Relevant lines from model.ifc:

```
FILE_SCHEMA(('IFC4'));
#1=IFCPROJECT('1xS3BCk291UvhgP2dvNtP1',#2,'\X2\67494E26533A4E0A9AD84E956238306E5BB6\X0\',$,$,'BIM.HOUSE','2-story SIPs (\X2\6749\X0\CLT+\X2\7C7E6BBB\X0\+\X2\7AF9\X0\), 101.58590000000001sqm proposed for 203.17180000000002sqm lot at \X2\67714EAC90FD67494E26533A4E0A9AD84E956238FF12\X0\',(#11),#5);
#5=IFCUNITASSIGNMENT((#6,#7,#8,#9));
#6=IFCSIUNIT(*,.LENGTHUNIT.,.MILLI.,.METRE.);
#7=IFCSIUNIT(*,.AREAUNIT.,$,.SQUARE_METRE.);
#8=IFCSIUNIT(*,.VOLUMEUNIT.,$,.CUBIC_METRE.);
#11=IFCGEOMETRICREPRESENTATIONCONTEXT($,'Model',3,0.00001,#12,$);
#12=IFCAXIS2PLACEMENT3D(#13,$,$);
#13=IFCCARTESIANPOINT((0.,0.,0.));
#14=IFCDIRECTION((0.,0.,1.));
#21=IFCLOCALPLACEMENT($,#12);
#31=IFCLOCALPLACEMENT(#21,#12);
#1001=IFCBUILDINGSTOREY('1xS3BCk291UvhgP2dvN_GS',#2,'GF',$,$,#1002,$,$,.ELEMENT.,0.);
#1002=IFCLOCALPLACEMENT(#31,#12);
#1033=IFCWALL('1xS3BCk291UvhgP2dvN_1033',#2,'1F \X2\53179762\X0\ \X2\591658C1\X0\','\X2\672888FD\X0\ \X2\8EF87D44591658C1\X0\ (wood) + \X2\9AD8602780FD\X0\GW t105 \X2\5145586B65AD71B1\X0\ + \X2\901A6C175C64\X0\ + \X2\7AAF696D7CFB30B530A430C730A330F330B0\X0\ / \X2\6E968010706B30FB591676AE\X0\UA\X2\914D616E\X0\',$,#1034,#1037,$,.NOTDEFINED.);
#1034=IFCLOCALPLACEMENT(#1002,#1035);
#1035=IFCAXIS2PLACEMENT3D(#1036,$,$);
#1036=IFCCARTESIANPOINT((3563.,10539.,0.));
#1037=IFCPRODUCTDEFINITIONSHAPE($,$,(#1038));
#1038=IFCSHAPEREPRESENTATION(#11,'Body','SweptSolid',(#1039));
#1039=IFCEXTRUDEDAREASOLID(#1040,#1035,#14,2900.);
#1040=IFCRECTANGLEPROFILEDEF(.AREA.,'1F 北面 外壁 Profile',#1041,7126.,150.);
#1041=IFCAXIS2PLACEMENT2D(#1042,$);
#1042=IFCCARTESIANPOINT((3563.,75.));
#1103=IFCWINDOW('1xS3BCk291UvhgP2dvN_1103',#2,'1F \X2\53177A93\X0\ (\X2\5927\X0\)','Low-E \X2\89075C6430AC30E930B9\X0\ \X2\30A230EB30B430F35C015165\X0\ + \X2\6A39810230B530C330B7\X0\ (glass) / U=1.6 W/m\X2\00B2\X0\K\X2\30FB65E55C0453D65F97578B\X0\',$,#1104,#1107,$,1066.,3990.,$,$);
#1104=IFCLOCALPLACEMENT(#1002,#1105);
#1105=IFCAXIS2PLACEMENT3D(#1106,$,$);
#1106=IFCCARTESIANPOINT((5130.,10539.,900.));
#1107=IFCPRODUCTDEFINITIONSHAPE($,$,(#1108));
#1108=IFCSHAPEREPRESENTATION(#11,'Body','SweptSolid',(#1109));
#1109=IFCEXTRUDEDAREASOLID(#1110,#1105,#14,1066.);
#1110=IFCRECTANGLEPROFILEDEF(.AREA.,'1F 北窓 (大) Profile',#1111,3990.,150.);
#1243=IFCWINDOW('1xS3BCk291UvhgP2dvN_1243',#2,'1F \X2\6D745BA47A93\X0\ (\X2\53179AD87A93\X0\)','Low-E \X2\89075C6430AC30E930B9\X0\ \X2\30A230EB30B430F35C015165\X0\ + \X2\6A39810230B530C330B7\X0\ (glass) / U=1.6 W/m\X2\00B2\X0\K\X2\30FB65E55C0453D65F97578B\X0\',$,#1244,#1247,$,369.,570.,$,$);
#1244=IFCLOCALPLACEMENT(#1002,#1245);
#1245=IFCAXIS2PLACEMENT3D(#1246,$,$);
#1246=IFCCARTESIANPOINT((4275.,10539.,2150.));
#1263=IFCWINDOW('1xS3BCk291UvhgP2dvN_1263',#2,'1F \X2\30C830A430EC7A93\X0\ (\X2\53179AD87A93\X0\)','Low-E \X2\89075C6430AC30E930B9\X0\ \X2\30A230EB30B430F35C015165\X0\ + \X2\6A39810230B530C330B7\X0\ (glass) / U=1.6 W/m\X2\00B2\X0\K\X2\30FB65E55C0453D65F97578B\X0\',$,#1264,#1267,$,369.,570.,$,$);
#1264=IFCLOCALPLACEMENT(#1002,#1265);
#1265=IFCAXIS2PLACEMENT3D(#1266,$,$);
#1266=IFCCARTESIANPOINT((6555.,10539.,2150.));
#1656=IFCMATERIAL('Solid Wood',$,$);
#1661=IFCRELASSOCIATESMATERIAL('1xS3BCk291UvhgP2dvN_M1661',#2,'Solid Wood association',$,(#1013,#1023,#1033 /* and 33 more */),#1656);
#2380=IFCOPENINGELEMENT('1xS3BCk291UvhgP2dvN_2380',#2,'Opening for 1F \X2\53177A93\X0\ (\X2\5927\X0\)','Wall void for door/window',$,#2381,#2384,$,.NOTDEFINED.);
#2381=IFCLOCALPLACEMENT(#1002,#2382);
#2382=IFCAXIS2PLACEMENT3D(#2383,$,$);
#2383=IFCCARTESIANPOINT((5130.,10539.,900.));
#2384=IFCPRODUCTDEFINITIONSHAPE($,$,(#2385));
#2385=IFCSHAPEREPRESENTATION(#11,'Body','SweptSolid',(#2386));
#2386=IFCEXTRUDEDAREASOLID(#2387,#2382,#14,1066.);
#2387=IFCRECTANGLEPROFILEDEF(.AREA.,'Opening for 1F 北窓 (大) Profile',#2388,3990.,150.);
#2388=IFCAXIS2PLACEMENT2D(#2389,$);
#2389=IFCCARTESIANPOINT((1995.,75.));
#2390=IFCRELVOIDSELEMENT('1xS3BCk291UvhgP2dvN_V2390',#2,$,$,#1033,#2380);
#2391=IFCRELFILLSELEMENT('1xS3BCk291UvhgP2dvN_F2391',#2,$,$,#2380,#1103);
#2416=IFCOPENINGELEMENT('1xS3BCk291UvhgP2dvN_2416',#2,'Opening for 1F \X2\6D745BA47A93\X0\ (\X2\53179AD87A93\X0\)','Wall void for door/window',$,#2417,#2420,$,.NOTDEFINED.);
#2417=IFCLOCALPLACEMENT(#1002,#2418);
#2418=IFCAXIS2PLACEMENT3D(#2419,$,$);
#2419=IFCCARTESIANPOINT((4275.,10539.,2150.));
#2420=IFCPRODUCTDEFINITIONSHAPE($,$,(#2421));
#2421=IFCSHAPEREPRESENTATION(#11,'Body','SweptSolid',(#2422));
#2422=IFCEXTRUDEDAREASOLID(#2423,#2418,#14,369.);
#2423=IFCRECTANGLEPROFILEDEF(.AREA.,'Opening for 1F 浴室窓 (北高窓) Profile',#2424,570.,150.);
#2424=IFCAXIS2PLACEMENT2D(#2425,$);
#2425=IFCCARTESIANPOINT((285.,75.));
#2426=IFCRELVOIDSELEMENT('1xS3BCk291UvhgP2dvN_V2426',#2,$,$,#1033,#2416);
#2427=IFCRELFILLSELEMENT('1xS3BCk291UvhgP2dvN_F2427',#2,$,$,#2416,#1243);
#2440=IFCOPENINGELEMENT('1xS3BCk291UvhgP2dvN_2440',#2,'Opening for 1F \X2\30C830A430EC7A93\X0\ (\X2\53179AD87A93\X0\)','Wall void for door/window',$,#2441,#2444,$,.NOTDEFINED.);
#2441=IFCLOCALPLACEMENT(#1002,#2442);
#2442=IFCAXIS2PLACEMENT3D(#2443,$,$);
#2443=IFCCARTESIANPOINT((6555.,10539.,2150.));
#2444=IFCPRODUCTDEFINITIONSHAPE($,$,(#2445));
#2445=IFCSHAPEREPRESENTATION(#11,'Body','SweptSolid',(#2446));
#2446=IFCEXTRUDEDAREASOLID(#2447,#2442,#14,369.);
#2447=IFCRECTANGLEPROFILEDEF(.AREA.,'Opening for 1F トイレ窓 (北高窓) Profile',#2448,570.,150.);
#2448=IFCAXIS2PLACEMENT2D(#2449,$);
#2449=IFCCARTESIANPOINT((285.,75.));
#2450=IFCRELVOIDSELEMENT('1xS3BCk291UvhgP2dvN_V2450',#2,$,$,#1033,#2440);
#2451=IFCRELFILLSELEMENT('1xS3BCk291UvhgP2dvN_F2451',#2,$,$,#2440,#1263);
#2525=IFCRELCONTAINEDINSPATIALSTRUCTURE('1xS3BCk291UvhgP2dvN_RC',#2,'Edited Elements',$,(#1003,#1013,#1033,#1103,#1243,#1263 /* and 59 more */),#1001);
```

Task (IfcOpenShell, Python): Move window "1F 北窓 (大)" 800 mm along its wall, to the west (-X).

```python
import ifcopenshell
import ifcopenshell.api.geometry
import ifcopenshell.util.placement

model = ifcopenshell.open("model.ifc")

window = model.by_guid("1xS3BCk291UvhgP2dvN_1103")
opening = window.FillsVoids[0].RelatingOpeningElement
wall = opening.VoidsElements[0].RelatingBuildingElement

wall_matrix = ifcopenshell.util.placement.get_local_placement(wall.ObjectPlacement)
shift = wall_matrix[:3, 0] * -800.0
before = ifcopenshell.util.placement.get_local_placement(window.ObjectPlacement)[:3, 3].copy()

# The window is not placed relative to its opening, so move both.
for product in (opening, window):
    matrix = ifcopenshell.util.placement.get_local_placement(product.ObjectPlacement)
    matrix[:3, 3] += shift
    ifcopenshell.api.geometry.edit_object_placement(model, product=product, matrix=matrix, is_si=False)

after = ifcopenshell.util.placement.get_local_placement(window.ObjectPlacement)[:3, 3]
print("window moved by", (after - before).round(3) + 0.0)

model.write("model_rev.ifc")
```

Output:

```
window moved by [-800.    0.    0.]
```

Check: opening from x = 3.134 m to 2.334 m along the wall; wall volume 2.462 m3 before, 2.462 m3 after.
